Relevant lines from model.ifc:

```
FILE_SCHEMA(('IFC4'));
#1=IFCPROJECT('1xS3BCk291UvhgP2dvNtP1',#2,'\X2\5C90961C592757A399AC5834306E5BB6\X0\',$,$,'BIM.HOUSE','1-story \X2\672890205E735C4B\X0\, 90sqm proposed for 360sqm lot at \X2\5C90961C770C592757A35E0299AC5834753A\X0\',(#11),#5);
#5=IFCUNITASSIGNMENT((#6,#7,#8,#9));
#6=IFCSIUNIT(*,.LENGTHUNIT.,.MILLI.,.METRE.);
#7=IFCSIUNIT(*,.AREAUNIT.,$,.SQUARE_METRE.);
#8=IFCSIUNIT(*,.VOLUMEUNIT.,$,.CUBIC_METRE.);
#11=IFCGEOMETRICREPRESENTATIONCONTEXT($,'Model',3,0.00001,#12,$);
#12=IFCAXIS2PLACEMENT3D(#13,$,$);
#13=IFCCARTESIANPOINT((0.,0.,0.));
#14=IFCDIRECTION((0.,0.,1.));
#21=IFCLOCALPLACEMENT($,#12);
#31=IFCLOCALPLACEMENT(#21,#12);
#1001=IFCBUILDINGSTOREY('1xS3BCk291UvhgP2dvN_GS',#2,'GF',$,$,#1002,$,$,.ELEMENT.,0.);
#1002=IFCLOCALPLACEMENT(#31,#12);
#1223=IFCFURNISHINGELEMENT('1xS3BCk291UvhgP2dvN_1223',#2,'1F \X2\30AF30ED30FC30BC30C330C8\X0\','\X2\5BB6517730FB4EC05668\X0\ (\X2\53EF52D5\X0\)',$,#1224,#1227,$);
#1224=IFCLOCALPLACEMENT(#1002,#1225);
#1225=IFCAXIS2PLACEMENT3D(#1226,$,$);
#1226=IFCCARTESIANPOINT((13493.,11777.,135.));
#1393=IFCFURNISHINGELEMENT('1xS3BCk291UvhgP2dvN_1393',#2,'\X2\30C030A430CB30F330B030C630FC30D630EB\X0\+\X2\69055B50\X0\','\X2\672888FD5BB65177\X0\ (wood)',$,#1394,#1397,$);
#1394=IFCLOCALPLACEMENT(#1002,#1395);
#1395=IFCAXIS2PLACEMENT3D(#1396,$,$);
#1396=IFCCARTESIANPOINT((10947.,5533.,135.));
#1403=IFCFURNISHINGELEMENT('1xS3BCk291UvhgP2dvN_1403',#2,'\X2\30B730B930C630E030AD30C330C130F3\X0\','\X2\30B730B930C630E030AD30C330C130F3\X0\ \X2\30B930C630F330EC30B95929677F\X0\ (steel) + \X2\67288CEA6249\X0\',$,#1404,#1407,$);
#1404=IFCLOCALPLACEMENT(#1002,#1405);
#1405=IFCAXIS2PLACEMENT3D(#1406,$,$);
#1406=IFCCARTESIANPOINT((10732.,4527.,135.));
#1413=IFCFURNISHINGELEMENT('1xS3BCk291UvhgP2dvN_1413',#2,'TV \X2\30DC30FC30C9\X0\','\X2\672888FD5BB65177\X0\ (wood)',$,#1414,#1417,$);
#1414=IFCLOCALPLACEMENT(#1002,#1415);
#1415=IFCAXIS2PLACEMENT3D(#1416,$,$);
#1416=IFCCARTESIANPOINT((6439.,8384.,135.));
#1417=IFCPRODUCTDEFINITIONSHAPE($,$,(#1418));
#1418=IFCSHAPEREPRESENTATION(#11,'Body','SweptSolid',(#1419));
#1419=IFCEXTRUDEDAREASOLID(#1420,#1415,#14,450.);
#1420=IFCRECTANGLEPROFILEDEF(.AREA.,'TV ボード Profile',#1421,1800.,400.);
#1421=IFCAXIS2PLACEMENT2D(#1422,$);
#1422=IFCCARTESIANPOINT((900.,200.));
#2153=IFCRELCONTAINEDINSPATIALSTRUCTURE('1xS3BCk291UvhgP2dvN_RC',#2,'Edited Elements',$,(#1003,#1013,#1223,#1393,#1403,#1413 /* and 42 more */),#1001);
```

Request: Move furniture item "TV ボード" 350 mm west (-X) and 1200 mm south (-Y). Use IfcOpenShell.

```python
import ifcopenshell
import ifcopenshell.api.geometry
import ifcopenshell.util.placement
import ifcopenshell.util.unit

model = ifcopenshell.open("model.ifc")
unit_scale = ifcopenshell.util.unit.calculate_unit_scale(model)

item = model.by_guid("1xS3BCk291UvhgP2dvN_1413")
matrix = ifcopenshell.util.placement.get_local_placement(item.ObjectPlacement)
matrix[0, 3] -= 0.35 / unit_scale
matrix[1, 3] -= 1.2 / unit_scale
ifcopenshell.api.geometry.edit_object_placement(model, product=item, matrix=matrix, is_si=False)

print(ifcopenshell.util.placement.get_local_placement(item.ObjectPlacement).round(3) + 0.0)

model.write("model_v2.ifc")
```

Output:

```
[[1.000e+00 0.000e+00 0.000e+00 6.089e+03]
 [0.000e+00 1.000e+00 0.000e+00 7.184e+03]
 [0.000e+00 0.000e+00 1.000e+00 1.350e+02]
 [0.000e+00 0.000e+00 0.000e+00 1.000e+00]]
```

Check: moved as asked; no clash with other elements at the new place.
